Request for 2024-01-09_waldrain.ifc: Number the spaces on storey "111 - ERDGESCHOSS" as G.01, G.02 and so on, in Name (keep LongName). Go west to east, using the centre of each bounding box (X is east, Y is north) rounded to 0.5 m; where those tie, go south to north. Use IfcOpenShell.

First a look at what the model holds.

```python
import ifcopenshell
import ifcopenshell.util.element
import ifcopenshell.util.placement

model = ifcopenshell.open("2024-01-09_waldrain.ifc")
print(model.schema)
storey = next(s for s in model.by_type("IfcBuildingStorey") if s.Name == "111 - ERDGESCHOSS")
spaces = [e for e in ifcopenshell.util.element.get_decomposition(storey) if e.is_a("IfcSpace")]
for e in sorted(spaces, key=lambda e: e.id()):
    origin = ifcopenshell.util.placement.get_local_placement(e.ObjectPlacement)[:3, 3]
    print(e.id(), e.Name, e.LongName, origin.round(2) + 0.0, sep=" | ")
```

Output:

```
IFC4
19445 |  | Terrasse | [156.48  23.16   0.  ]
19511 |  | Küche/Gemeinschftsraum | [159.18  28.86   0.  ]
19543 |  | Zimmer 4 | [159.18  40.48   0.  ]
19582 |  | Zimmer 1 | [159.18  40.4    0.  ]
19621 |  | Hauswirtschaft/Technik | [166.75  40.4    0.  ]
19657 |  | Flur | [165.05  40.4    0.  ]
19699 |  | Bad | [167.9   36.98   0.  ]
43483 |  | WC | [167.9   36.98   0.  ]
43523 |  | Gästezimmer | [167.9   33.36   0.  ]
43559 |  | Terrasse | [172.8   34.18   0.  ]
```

```python
import ifcopenshell
import ifcopenshell.geom
import ifcopenshell.util.element
import ifcopenshell.util.shape

model = ifcopenshell.open("2024-01-09_waldrain.ifc")
settings = ifcopenshell.geom.settings()
settings.set("use-world-coords", True)


def centre(element):
    shape = ifcopenshell.geom.create_shape(settings, element)
    return ifcopenshell.util.shape.get_bbox_centroid(shape.geometry)


storey = next(s for s in model.by_type("IfcBuildingStorey") if s.Name == "111 - ERDGESCHOSS")
spaces = [e for e in ifcopenshell.util.element.get_decomposition(storey) if e.is_a("IfcSpace")]

# Insertion points can sit at a corner or the storey origin, so sort by the geometry (in metres).
centres = {e: centre(e) for e in spaces}
spaces.sort(key=lambda e: (round(centres[e][0] / 0.5), centres[e][1]))

for i, e in enumerate(spaces, start=1):
    number = f"G.{i:02d}"
    e.Name = number
    print(e.id(), number)

model.write("2024-01-09_waldrain_rev.ifc")
```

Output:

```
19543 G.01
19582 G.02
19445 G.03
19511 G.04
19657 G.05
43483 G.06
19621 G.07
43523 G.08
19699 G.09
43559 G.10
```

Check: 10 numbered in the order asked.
